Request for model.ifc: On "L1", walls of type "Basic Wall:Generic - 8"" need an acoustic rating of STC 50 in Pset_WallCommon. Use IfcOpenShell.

First a look at what the model holds.

```python
import ifcopenshell
import ifcopenshell.util.element

model = ifcopenshell.open("model.ifc")
print(model.schema)
storey = next(s for s in model.by_type("IfcBuildingStorey") if s.Name == "L1")
walls = [e for e in ifcopenshell.util.element.get_decomposition(storey) if e.is_a("IfcWall")]
seen = {}
for e in walls:
    element_type = ifcopenshell.util.element.get_type(e)
    key = (element_type.Name if element_type != e and element_type else None, ifcopenshell.util.element.get_pset(e, "Pset_WallCommon", "AcousticRating"))
    seen[key] = seen.get(key, 0) + 1
for (name, value), count in sorted(seen.items(), key=str):
    print(count, "x", name, "|", value)
```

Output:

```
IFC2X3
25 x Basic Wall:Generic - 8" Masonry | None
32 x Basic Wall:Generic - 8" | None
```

```python
import ifcopenshell
import ifcopenshell.api.pset
import ifcopenshell.util.element

model = ifcopenshell.open("model.ifc")

storey = next(s for s in model.by_type("IfcBuildingStorey") if s.Name == "L1")
walls = [e for e in ifcopenshell.util.element.get_decomposition(storey) if e.is_a("IfcWall")]

count = 0
for e in walls:
    element_type = ifcopenshell.util.element.get_type(e)
    if element_type in (None, e) or element_type.Name != 'Basic Wall:Generic - 8"':
        continue
    # add_pset returns the element's existing set when there is one.
    pset = ifcopenshell.api.pset.add_pset(model, product=e, name="Pset_WallCommon")
    ifcopenshell.api.pset.edit_pset(model, pset=pset, properties={"AcousticRating": "STC 50"})
    count += 1

print(count, "walls updated")

model.write("model_rev.ifc")
```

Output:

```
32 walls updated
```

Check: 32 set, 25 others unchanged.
